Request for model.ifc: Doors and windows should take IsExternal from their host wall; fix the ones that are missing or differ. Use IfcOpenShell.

First a look at what the model holds.

```python
import ifcopenshell
import ifcopenshell.util.element

model = ifcopenshell.open("model.ifc")
print(model.schema)
seen = {}
for e in model.by_type("IfcDoor") + model.by_type("IfcWindow"):
    if not e.FillsVoids:
        continue
    host = e.FillsVoids[0].RelatingOpeningElement.VoidsElements[0].RelatingBuildingElement
    own = ifcopenshell.util.element.get_pset(e, f"Pset_{e.is_a()[3:].removesuffix('StandardCase')}Common", "IsExternal")
    wall = ifcopenshell.util.element.get_pset(host, "Pset_WallCommon", "IsExternal")
    seen[e.is_a(), own, wall] = seen.get((e.is_a(), own, wall), 0) + 1
for (cls, own, wall), count in sorted(seen.items(), key=str):
    print(count, cls, "IsExternal:", own, "| host wall:", wall)
```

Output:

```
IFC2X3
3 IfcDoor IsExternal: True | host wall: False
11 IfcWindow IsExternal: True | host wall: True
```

```python
import ifcopenshell
import ifcopenshell.api.pset
import ifcopenshell.util.element

model = ifcopenshell.open("model.ifc")

count = 0
for ifc_class, pset_name in (("IfcDoor", "Pset_DoorCommon"), ("IfcWindow", "Pset_WindowCommon")):
    for e in model.by_type(ifc_class):
        if not e.FillsVoids:
            continue
        host = e.FillsVoids[0].RelatingOpeningElement.VoidsElements[0].RelatingBuildingElement
        external = ifcopenshell.util.element.get_pset(host, "Pset_WallCommon", "IsExternal")
        if external is None or ifcopenshell.util.element.get_pset(e, pset_name, "IsExternal") == external:
            continue
        pset = ifcopenshell.api.pset.add_pset(model, product=e, name=pset_name)
        ifcopenshell.api.pset.edit_pset(model, pset=pset, properties={"IsExternal": external})
        count += 1

print(count, "updated")

model.write("model_updated.ifc")
```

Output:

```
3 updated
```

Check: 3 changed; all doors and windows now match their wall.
